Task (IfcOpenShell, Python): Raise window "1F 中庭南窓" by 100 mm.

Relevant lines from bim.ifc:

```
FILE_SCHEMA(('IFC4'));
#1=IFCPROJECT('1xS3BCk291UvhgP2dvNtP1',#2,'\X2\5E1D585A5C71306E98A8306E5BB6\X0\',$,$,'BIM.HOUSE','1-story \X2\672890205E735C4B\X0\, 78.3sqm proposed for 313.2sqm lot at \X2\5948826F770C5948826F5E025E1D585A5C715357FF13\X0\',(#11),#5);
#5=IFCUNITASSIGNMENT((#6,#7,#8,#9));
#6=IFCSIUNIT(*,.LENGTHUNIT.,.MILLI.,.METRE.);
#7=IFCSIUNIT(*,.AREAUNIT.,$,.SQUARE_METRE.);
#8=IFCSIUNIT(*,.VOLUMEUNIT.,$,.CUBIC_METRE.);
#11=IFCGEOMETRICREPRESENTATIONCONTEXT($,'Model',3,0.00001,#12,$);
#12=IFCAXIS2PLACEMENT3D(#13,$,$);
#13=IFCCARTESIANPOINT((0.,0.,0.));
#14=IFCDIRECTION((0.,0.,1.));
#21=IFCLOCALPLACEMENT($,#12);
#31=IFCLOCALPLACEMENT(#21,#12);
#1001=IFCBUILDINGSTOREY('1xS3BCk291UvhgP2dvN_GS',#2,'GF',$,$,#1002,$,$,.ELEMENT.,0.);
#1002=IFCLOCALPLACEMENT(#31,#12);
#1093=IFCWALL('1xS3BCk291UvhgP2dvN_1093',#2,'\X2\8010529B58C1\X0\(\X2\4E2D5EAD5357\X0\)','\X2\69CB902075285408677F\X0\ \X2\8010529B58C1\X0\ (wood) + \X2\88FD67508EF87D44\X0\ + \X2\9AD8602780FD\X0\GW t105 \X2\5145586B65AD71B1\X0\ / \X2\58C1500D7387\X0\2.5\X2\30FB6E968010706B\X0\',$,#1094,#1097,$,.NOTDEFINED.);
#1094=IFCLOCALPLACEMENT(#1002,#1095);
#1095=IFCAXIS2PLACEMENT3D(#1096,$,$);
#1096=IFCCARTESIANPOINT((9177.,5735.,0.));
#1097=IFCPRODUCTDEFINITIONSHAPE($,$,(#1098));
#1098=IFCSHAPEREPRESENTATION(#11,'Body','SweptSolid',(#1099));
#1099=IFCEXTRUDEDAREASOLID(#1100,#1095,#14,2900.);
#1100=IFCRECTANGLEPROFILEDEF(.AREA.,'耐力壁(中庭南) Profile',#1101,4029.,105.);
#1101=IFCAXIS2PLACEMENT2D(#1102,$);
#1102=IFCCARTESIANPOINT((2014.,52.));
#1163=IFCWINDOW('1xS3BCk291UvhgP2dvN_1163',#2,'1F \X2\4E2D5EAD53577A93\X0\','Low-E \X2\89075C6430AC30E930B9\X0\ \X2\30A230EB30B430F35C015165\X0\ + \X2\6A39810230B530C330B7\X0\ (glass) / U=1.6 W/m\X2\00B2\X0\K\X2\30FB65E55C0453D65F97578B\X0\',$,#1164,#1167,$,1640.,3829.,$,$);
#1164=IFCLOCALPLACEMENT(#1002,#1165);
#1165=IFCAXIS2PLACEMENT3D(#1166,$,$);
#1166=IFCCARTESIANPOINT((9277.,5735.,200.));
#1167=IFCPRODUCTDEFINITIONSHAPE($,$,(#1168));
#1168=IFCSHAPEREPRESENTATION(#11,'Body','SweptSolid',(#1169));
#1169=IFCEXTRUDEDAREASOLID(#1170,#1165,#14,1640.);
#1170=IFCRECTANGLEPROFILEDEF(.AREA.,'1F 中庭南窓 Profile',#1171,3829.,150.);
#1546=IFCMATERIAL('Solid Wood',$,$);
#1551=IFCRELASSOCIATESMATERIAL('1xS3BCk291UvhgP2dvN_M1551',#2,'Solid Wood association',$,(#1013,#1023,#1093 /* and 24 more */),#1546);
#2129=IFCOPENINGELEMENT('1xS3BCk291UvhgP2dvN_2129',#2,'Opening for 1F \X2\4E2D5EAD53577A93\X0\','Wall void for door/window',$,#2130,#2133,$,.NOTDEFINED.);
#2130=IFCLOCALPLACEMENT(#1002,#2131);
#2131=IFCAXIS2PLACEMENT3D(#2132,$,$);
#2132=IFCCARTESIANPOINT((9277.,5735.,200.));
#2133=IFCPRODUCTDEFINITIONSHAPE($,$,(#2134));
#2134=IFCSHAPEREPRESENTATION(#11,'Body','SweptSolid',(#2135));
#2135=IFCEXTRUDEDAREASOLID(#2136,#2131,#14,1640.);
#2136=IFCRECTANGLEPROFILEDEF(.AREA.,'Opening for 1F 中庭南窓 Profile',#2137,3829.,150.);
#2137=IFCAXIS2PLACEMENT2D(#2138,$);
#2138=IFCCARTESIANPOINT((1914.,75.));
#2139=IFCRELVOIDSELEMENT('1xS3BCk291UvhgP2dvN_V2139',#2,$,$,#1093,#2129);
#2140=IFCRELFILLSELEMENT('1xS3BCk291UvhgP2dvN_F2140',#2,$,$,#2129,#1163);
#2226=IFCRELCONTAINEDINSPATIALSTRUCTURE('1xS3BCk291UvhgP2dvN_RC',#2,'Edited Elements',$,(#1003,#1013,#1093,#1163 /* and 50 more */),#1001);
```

```python
import numpy as np
import ifcopenshell
import ifcopenshell.api.geometry
import ifcopenshell.util.placement
import ifcopenshell.util.unit

model = ifcopenshell.open("bim.ifc")
unit_scale = ifcopenshell.util.unit.calculate_unit_scale(model)

window = model.by_guid("1xS3BCk291UvhgP2dvN_1163")
opening = window.FillsVoids[0].RelatingOpeningElement
dz = 100.0

shift = np.array([0.0, 0.0, dz])
# The window is not placed relative to its opening, so move both.
for product in (opening, window):
    matrix = ifcopenshell.util.placement.get_local_placement(product.ObjectPlacement)
    matrix[:3, 3] += shift
    ifcopenshell.api.geometry.edit_object_placement(model, product=product, matrix=matrix, is_si=False)

print(f"moved by {dz * unit_scale:+.3f} m")

model.write("bim_updated.ifc")
```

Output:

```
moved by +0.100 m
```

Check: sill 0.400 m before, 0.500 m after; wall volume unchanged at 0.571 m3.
